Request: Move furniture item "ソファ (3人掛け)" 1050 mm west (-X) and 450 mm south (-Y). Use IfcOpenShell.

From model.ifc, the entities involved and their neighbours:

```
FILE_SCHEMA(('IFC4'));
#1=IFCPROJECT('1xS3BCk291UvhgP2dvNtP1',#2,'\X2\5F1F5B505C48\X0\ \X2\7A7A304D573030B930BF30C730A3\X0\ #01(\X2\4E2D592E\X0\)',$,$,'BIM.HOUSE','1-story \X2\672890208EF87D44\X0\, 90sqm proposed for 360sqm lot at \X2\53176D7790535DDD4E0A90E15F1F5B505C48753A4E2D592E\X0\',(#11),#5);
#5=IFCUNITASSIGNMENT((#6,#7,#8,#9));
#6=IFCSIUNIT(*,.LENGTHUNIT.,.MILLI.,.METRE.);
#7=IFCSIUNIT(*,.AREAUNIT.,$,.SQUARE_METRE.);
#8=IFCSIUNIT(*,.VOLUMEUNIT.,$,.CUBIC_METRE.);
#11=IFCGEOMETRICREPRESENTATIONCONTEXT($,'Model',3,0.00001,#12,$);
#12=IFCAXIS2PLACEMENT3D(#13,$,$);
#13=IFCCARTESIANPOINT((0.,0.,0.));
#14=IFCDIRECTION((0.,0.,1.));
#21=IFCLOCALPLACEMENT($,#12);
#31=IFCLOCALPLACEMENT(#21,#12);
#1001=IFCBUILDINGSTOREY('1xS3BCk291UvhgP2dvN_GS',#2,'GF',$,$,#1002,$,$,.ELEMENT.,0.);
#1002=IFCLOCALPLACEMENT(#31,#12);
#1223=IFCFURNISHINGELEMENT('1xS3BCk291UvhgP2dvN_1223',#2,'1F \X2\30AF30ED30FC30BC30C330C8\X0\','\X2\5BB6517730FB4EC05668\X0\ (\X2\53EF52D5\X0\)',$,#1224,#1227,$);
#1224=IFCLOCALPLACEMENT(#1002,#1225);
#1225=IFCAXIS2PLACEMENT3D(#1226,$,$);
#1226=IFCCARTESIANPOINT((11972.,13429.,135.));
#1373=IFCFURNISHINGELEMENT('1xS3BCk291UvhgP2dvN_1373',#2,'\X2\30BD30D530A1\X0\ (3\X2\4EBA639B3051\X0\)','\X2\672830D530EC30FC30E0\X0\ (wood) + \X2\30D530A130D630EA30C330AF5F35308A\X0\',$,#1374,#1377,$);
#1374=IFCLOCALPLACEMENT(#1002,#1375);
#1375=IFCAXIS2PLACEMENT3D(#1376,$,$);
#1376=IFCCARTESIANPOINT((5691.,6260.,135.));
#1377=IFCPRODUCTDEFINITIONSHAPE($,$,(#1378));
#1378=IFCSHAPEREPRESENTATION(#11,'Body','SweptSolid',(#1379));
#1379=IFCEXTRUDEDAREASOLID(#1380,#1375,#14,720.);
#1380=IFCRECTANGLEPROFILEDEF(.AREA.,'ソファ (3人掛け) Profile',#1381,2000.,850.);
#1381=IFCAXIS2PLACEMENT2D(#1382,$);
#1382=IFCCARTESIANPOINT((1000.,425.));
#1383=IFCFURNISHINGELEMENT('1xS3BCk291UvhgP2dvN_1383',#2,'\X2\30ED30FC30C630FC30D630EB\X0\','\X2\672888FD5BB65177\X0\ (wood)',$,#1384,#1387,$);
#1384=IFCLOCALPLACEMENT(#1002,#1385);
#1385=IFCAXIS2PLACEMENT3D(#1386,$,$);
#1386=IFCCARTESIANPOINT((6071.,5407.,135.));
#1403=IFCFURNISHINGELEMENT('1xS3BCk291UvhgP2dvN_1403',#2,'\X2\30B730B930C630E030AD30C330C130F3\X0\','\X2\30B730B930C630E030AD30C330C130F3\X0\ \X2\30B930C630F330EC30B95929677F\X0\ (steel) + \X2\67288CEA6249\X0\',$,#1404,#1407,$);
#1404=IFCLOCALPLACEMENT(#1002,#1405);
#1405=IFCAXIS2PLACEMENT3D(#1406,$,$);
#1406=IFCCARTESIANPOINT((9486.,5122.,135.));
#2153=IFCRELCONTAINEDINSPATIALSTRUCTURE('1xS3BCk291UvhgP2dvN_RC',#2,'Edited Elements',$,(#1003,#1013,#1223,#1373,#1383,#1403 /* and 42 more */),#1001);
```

```python
import ifcopenshell
import ifcopenshell.api.geometry
import ifcopenshell.util.placement

model = ifcopenshell.open("model.ifc")

item = model.by_guid("1xS3BCk291UvhgP2dvN_1373")
matrix = ifcopenshell.util.placement.get_local_placement(item.ObjectPlacement)
matrix[0, 3] -= 1050.0
matrix[1, 3] -= 450.0
ifcopenshell.api.geometry.edit_object_placement(model, product=item, matrix=matrix, is_si=False)

print(ifcopenshell.util.placement.get_local_placement(item.ObjectPlacement).round(3) + 0.0)

model.write("model_edited.ifc")
```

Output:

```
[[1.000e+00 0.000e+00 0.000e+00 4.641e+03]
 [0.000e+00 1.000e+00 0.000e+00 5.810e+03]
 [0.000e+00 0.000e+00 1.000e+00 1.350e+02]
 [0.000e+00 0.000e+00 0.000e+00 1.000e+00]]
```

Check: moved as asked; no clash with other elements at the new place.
